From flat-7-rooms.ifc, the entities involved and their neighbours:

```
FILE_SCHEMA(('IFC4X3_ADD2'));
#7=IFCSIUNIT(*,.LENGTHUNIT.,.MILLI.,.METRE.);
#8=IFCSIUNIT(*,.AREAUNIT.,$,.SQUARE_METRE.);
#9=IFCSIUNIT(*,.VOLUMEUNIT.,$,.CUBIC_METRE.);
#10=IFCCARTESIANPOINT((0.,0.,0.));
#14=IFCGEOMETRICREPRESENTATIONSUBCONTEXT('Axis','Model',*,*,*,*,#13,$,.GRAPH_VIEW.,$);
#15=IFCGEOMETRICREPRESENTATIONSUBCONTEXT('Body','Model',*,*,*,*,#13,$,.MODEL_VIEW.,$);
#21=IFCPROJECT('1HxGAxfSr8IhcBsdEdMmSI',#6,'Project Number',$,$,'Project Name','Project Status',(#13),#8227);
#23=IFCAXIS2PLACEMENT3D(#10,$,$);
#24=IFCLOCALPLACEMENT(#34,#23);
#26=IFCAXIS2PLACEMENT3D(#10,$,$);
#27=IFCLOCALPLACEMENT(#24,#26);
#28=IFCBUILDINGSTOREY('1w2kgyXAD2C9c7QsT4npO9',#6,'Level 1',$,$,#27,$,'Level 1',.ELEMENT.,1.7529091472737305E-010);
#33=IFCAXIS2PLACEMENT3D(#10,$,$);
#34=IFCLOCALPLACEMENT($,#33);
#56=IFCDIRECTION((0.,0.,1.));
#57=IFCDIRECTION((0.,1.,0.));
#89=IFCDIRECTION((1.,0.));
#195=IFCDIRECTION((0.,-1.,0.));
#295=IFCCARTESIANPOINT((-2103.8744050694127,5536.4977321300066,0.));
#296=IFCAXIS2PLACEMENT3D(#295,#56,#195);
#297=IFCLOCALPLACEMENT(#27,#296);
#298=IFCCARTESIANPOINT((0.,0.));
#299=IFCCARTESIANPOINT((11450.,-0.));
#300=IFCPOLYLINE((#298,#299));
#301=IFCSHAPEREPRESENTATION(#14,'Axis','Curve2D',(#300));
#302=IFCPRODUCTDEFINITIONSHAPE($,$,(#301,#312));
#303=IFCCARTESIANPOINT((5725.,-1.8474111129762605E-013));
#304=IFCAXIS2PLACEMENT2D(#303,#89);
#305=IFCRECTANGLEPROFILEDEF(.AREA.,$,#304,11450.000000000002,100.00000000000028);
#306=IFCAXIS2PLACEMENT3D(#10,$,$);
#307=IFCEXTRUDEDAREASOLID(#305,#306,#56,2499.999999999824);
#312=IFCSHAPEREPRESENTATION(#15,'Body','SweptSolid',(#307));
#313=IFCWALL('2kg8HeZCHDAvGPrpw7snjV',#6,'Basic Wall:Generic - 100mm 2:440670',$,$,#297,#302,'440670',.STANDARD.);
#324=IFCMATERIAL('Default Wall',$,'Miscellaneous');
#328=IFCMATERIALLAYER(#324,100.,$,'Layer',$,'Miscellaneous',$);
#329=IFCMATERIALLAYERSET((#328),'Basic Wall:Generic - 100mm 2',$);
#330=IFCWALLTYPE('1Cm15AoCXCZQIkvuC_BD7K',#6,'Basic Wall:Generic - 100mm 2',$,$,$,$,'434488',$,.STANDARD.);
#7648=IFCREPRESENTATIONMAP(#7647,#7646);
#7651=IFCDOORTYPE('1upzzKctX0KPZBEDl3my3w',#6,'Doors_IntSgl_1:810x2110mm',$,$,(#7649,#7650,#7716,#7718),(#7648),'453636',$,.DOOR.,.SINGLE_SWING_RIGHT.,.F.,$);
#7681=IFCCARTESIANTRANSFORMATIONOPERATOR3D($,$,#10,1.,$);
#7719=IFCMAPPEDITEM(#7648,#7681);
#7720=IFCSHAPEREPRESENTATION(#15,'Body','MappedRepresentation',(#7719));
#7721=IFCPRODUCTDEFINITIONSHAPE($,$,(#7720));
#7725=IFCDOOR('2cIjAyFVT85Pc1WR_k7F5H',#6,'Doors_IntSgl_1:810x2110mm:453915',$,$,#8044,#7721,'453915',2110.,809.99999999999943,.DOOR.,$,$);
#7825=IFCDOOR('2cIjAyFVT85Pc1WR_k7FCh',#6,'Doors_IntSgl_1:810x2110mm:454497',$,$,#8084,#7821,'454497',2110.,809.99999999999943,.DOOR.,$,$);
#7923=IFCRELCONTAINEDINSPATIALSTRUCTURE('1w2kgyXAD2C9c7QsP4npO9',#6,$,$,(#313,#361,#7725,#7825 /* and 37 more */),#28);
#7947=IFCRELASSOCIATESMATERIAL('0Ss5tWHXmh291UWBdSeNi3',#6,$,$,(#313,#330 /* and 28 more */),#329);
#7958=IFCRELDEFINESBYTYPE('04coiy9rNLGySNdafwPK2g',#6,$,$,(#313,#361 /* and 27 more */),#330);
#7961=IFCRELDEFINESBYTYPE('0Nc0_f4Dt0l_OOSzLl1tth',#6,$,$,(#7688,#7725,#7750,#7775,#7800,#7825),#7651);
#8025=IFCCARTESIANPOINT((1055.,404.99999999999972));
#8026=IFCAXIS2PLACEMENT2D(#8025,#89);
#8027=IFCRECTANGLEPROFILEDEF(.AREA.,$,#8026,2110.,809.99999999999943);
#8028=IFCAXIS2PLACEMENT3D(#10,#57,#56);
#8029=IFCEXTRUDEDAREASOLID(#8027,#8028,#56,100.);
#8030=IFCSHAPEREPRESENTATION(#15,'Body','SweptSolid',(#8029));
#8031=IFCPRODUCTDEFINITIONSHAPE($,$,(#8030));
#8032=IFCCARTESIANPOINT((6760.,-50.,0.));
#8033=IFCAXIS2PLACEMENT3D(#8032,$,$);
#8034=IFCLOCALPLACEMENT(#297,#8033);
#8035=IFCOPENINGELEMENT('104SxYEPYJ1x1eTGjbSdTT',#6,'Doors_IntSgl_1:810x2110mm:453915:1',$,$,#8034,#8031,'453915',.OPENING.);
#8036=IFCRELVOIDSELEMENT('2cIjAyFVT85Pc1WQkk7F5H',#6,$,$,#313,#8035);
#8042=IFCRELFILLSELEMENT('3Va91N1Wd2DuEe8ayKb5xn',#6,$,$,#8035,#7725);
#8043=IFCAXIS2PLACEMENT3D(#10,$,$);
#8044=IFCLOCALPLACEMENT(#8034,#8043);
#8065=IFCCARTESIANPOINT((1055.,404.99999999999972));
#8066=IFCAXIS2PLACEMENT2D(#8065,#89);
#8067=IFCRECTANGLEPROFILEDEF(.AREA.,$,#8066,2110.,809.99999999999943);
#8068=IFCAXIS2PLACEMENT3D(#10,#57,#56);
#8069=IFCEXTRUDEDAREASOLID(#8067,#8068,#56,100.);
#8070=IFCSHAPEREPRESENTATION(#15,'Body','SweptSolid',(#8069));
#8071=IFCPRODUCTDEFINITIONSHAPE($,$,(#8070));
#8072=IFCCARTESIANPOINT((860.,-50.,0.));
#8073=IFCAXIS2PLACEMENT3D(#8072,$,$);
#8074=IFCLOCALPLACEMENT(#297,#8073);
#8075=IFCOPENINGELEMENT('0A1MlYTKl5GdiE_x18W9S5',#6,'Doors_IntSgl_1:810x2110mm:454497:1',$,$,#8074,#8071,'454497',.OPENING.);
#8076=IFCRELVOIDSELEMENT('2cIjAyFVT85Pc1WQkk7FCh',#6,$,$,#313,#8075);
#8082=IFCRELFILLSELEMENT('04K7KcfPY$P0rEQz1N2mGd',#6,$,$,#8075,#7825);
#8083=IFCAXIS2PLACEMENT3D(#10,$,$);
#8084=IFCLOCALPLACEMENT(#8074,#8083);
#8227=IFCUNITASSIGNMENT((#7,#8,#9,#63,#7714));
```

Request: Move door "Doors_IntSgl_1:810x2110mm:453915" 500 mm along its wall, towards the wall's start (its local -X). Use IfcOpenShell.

```python
import ifcopenshell
import ifcopenshell.api.geometry
import ifcopenshell.util.placement
import ifcopenshell.util.unit

model = ifcopenshell.open("flat-7-rooms.ifc")
unit_scale = ifcopenshell.util.unit.calculate_unit_scale(model)

door = model.by_id(7725)
opening = door.FillsVoids[0].RelatingOpeningElement
wall = opening.VoidsElements[0].RelatingBuildingElement

wall_matrix = ifcopenshell.util.placement.get_local_placement(wall.ObjectPlacement)
shift = wall_matrix[:3, 0] * -0.5 / unit_scale
before = ifcopenshell.util.placement.get_local_placement(door.ObjectPlacement)[:3, 3].copy()

# The door is placed relative to its opening, so it follows when the opening moves.
matrix = ifcopenshell.util.placement.get_local_placement(opening.ObjectPlacement)
matrix[:3, 3] += shift
ifcopenshell.api.geometry.edit_object_placement(
    model, product=opening, matrix=matrix, is_si=False, should_transform_children=True
)

after = ifcopenshell.util.placement.get_local_placement(door.ObjectPlacement)[:3, 3]
print("door moved by", (after - before).round(3) + 0.0)

model.write("flat-7-rooms_v2.ifc")
```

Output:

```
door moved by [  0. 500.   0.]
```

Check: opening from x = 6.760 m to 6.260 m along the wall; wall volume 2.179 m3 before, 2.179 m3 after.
